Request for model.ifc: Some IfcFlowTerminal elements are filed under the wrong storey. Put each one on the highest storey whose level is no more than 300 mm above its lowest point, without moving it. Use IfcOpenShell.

First a look at what the model holds.

```python
import ifcopenshell
import ifcopenshell.util.element
import ifcopenshell.util.placement

model = ifcopenshell.open("model.ifc")
print(model.schema)
for storey in model.by_type("IfcBuildingStorey"):
    level = ifcopenshell.util.placement.get_storey_elevation(storey)
    count = sum(e.is_a("IfcFlowTerminal") for e in ifcopenshell.util.element.get_contained(storey))
    print(storey.id(), storey.Name, round(level, 3), count, sep=" | ")
```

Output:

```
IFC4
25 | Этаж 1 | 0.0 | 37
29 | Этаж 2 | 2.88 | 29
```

```python
import ifcopenshell
import ifcopenshell.api.spatial
import ifcopenshell.geom
import ifcopenshell.util.element
import ifcopenshell.util.placement
import ifcopenshell.util.shape
import ifcopenshell.util.unit

model = ifcopenshell.open("model.ifc")
unit_scale = ifcopenshell.util.unit.calculate_unit_scale(model)
settings = ifcopenshell.geom.settings()

levels = sorted(
    ((ifcopenshell.util.placement.get_storey_elevation(s) * unit_scale, s) for s in model.by_type("IfcBuildingStorey")),
    key=lambda pair: pair[0],
)

for e in model.by_type("IfcFlowTerminal"):
    current = e.ContainedInStructure[0].RelatingStructure if e.ContainedInStructure else None
    if current is None or not current.is_a("IfcBuildingStorey"):
        continue
    shape = ifcopenshell.geom.create_shape(settings, e)
    bottom = ifcopenshell.util.shape.get_shape_bottom_elevation(shape, shape.geometry)
    below = [s for level, s in levels if level <= bottom + 0.3]
    storey = below[-1] if below else levels[0][1]
    if storey != current:
        # assign_container keeps the world position.
        ifcopenshell.api.spatial.assign_container(model, products=[e], relating_structure=storey)
        print(e.id(), current.Name, "->", storey.Name)

model.write("model_v2.ifc")
```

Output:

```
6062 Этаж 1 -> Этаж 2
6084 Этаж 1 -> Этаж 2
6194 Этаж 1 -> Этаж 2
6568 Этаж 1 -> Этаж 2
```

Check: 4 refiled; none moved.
